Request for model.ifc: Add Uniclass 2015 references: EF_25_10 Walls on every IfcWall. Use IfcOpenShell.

First a look at what the model holds.

```python
import ifcopenshell

model = ifcopenshell.open("model.ifc")
print(model.schema)
print("classifications:", [c.Name for c in model.by_type("IfcClassification")])
for ifc_class in ("IfcDoor", "IfcRoof", "IfcStair", "IfcWall", "IfcWindow"):
    print(ifc_class, len(model.by_type(ifc_class)))
```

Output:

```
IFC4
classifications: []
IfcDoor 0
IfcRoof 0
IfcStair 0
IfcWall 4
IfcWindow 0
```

```python
import ifcopenshell
import ifcopenshell.api.classification

model = ifcopenshell.open("model.ifc")

system = ifcopenshell.api.classification.add_classification(model, classification="Uniclass 2015")

codes = {
    "IfcWall": ("EF_25_10", "Walls"),
}
for ifc_class, (code, name) in codes.items():
    products = model.by_type(ifc_class)
    ifcopenshell.api.classification.add_reference(
        model, products=products, classification=system, identification=code, name=name
    )
    print(code, len(products))

model.write("model-out.ifc")
```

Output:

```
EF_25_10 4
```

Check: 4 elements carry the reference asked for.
